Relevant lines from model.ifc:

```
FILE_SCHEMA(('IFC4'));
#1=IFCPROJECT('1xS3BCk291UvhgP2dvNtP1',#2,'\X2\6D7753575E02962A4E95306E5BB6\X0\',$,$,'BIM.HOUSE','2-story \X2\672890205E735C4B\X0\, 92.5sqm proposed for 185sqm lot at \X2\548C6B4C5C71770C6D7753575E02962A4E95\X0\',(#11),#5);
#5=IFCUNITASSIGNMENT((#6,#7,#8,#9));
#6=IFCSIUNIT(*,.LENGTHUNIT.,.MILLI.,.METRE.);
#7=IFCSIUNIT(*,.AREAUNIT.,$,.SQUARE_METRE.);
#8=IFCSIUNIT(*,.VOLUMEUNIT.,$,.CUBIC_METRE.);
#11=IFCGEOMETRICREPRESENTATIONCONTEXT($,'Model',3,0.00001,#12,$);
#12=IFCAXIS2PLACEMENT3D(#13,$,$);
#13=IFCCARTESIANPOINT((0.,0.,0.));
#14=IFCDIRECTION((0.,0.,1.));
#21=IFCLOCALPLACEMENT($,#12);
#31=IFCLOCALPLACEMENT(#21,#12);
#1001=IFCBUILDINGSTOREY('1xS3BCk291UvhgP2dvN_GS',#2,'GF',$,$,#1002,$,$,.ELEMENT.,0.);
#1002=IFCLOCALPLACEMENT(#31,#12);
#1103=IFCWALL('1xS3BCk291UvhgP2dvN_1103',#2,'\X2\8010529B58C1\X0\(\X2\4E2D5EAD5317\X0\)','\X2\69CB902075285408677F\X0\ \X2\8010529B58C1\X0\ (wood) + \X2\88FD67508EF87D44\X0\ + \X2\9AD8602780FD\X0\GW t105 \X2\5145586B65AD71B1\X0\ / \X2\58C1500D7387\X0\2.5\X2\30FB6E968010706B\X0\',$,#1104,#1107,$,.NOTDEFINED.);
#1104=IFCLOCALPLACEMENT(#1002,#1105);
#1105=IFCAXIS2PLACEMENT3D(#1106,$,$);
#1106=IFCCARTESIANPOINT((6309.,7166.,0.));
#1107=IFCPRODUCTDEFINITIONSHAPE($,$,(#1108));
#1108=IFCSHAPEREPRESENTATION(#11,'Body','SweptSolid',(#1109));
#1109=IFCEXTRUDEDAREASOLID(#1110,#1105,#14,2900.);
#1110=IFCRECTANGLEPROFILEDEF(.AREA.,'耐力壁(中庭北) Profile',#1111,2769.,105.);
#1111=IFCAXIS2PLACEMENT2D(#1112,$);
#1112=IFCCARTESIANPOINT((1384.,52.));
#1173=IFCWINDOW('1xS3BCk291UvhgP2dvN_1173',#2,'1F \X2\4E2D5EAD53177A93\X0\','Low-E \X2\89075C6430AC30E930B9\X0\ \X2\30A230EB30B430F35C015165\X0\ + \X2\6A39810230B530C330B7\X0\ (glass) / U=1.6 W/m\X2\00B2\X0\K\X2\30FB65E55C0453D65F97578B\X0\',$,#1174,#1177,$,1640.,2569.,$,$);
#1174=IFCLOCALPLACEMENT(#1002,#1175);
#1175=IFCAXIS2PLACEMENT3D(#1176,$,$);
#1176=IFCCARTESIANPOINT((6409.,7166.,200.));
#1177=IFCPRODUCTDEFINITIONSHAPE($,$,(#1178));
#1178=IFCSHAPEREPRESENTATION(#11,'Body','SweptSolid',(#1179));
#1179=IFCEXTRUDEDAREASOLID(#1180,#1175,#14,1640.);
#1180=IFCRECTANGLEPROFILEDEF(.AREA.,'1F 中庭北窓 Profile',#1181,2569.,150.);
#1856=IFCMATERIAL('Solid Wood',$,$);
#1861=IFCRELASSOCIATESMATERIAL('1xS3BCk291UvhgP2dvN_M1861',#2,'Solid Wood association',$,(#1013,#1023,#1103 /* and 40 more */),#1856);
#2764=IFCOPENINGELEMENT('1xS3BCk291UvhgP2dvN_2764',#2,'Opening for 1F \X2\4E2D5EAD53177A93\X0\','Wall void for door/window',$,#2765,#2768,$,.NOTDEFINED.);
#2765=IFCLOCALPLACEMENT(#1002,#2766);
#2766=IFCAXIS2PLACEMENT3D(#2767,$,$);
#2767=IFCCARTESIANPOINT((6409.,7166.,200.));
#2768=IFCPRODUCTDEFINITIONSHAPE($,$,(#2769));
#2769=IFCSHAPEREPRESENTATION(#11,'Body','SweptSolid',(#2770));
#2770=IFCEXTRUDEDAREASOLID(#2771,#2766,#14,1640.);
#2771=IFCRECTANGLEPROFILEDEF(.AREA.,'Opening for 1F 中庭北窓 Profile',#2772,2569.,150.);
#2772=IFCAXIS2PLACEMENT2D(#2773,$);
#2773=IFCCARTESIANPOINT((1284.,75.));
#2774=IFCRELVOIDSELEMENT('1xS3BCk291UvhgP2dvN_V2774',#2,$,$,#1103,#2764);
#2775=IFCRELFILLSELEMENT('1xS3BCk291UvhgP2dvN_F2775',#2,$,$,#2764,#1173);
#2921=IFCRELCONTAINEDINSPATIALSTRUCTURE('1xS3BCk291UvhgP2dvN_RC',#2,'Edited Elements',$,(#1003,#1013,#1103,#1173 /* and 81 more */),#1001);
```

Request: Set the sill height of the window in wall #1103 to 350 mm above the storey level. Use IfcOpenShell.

```python
import numpy as np
import ifcopenshell
import ifcopenshell.api.geometry
import ifcopenshell.geom
import ifcopenshell.util.element
import ifcopenshell.util.placement
import ifcopenshell.util.shape
import ifcopenshell.util.unit

model = ifcopenshell.open("model.ifc")
unit_scale = ifcopenshell.util.unit.calculate_unit_scale(model)

window = model.by_id(1173)
opening = window.FillsVoids[0].RelatingOpeningElement
storey = ifcopenshell.util.element.get_container(window, ifc_class="IfcBuildingStorey")
level = ifcopenshell.util.placement.get_local_placement(storey.ObjectPlacement)[2, 3]

# The opening's origin need not be at the sill, so measure its lowest point.
shape = ifcopenshell.geom.create_shape(ifcopenshell.geom.settings(), opening)
bottom = ifcopenshell.util.shape.get_shape_bottom_elevation(shape, shape.geometry) / unit_scale
dz = level + 0.35 / unit_scale - bottom

shift = np.array([0.0, 0.0, dz])
# The window is not placed relative to its opening, so move both.
for product in (opening, window):
    matrix = ifcopenshell.util.placement.get_local_placement(product.ObjectPlacement)
    matrix[:3, 3] += shift
    ifcopenshell.api.geometry.edit_object_placement(model, product=product, matrix=matrix, is_si=False)

print(f"moved by {dz * unit_scale:+.3f} m")

model.write("model_rev.ifc")
```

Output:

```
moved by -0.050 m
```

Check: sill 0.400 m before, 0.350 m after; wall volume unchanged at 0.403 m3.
